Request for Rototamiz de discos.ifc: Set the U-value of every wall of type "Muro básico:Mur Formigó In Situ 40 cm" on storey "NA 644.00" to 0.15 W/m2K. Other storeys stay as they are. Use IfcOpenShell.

First a look at what the model holds.

```python
import ifcopenshell
import ifcopenshell.util.element

model = ifcopenshell.open("Rototamiz de discos.ifc")
print(model.schema)
storey = next(s for s in model.by_type("IfcBuildingStorey") if s.Name == "NA 644.00")
walls = [e for e in ifcopenshell.util.element.get_decomposition(storey) if e.is_a("IfcWall")]
seen = {}
for e in walls:
    element_type = ifcopenshell.util.element.get_type(e)
    key = (element_type.Name if element_type != e and element_type else None, ifcopenshell.util.element.get_pset(e, "Pset_WallCommon", "ThermalTransmittance"))
    seen[key] = seen.get(key, 0) + 1
for (name, value), count in sorted(seen.items(), key=str):
    print(count, "x", name, "|", value)
```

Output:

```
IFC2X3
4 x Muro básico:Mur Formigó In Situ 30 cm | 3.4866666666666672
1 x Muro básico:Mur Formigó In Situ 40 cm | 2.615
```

```python
import ifcopenshell
import ifcopenshell.api.pset
import ifcopenshell.util.element

model = ifcopenshell.open("Rototamiz de discos.ifc")

storey = next(s for s in model.by_type("IfcBuildingStorey") if s.Name == "NA 644.00")
walls = [e for e in ifcopenshell.util.element.get_decomposition(storey) if e.is_a("IfcWall")]

count = 0
for e in walls:
    element_type = ifcopenshell.util.element.get_type(e)
    if element_type in (None, e) or element_type.Name != "Muro básico:Mur Formigó In Situ 40 cm":
        continue
    # add_pset returns the element's existing set when there is one.
    pset = ifcopenshell.api.pset.add_pset(model, product=e, name="Pset_WallCommon")
    ifcopenshell.api.pset.edit_pset(model, pset=pset, properties={"ThermalTransmittance": 0.15})
    count += 1

print(count, "walls updated")

model.write("Rototamiz de discos-out.ifc")
```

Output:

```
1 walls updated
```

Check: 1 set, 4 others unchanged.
